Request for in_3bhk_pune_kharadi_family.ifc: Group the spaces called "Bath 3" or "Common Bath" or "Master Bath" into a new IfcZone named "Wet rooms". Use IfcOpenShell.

First a look at what the model holds.

```python
import ifcopenshell

model = ifcopenshell.open("in_3bhk_pune_kharadi_family.ifc")
print(model.schema)
seen = {}
for space in model.by_type("IfcSpace"):
    seen[space.LongName] = seen.get(space.LongName, 0) + 1
for name, count in sorted(seen.items(), key=str):
    print(count, "x", name)
print("zones:", [z.Name for z in model.by_type("IfcZone")][:20])
```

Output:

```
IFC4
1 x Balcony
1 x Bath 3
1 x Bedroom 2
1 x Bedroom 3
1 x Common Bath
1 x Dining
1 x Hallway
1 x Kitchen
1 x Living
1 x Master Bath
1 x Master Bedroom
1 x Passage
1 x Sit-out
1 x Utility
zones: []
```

```python
import ifcopenshell
import ifcopenshell.api.group
import ifcopenshell.api.root

model = ifcopenshell.open("in_3bhk_pune_kharadi_family.ifc")

names = {"Bath 3", "Common Bath", "Master Bath"}
spaces = [s for s in model.by_type("IfcSpace") if s.LongName in names]

zone = ifcopenshell.api.root.create_entity(model, ifc_class="IfcZone", name="Wet rooms")
ifcopenshell.api.group.assign_group(model, products=spaces, group=zone)
print(len(spaces), "spaces in", zone.Name)

model.write("in_3bhk_pune_kharadi_family-out.ifc")
```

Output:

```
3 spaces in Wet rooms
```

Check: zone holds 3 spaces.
